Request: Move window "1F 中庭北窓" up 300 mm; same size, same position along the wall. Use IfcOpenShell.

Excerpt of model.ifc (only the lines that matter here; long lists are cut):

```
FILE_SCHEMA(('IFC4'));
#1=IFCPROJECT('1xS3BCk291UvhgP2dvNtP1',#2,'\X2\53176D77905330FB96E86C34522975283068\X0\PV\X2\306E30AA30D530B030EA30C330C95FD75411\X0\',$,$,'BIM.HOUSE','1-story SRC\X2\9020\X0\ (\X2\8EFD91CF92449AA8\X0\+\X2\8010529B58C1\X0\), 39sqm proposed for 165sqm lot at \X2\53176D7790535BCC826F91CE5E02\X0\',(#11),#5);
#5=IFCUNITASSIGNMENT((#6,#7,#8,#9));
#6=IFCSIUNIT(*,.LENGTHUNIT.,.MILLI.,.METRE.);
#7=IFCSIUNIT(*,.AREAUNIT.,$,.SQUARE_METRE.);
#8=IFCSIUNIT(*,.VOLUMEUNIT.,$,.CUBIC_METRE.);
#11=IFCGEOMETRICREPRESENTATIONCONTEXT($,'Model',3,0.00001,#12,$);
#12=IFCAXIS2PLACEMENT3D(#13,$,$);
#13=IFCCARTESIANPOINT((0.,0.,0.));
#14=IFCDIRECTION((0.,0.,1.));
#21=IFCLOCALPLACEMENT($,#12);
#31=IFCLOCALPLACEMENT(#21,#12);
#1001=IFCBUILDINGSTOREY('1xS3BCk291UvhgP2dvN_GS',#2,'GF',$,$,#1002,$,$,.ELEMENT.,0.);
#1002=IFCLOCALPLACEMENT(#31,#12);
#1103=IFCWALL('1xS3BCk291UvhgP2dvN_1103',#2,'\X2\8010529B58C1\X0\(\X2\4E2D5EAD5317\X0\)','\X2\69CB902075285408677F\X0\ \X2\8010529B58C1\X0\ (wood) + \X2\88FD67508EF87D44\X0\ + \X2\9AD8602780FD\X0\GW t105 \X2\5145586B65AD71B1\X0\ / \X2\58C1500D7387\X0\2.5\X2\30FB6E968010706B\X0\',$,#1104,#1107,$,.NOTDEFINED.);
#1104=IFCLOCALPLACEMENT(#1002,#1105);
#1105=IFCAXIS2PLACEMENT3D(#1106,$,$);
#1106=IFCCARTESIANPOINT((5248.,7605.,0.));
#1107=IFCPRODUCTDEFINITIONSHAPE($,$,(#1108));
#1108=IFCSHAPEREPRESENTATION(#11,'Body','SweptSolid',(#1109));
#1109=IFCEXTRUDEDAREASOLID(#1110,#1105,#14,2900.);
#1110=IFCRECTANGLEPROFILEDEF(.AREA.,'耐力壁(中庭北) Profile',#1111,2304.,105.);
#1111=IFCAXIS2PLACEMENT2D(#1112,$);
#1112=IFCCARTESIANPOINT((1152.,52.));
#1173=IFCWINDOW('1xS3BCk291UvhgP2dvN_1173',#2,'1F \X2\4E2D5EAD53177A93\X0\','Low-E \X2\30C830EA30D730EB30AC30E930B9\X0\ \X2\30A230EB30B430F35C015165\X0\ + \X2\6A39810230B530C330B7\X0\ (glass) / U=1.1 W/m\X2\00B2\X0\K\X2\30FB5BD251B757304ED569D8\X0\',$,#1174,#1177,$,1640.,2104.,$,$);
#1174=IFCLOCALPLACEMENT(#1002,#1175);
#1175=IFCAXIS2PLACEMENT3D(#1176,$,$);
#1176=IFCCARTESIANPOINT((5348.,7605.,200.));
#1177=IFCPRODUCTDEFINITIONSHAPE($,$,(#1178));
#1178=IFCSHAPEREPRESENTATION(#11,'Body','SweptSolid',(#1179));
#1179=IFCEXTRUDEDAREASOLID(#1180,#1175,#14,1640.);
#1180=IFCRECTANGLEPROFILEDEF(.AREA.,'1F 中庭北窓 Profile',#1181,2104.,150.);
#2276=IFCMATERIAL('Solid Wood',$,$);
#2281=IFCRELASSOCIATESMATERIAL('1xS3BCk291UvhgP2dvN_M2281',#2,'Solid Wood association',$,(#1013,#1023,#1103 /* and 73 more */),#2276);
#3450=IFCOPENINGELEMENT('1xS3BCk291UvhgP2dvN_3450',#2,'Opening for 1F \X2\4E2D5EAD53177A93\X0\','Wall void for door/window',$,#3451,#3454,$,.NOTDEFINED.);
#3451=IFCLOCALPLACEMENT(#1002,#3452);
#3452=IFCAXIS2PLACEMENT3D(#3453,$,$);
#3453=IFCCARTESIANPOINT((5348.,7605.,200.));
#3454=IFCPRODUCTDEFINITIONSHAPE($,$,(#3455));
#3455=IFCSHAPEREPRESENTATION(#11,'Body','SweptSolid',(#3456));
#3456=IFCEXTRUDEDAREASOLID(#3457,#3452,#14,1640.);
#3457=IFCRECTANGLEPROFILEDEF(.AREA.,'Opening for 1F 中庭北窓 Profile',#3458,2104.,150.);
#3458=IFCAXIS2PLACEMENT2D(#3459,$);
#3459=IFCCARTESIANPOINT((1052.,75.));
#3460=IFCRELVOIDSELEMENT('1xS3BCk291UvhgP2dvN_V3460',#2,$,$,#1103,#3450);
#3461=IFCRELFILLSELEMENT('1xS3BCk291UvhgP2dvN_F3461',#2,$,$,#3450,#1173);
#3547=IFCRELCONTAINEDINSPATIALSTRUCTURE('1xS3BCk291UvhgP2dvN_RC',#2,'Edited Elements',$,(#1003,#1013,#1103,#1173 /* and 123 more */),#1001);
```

```python
import numpy as np
import ifcopenshell
import ifcopenshell.api.geometry
import ifcopenshell.util.placement
import ifcopenshell.util.unit

model = ifcopenshell.open("model.ifc")
unit_scale = ifcopenshell.util.unit.calculate_unit_scale(model)

window = model.by_guid("1xS3BCk291UvhgP2dvN_1173")
opening = window.FillsVoids[0].RelatingOpeningElement
dz = 0.3 / unit_scale

shift = np.array([0.0, 0.0, dz])
# The window is not placed relative to its opening, so move both.
for product in (opening, window):
    matrix = ifcopenshell.util.placement.get_local_placement(product.ObjectPlacement)
    matrix[:3, 3] += shift
    ifcopenshell.api.geometry.edit_object_placement(model, product=product, matrix=matrix, is_si=False)

print(f"moved by {dz * unit_scale:+.3f} m")

model.write("model_updated.ifc")
```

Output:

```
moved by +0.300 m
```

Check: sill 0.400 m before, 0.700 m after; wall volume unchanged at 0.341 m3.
